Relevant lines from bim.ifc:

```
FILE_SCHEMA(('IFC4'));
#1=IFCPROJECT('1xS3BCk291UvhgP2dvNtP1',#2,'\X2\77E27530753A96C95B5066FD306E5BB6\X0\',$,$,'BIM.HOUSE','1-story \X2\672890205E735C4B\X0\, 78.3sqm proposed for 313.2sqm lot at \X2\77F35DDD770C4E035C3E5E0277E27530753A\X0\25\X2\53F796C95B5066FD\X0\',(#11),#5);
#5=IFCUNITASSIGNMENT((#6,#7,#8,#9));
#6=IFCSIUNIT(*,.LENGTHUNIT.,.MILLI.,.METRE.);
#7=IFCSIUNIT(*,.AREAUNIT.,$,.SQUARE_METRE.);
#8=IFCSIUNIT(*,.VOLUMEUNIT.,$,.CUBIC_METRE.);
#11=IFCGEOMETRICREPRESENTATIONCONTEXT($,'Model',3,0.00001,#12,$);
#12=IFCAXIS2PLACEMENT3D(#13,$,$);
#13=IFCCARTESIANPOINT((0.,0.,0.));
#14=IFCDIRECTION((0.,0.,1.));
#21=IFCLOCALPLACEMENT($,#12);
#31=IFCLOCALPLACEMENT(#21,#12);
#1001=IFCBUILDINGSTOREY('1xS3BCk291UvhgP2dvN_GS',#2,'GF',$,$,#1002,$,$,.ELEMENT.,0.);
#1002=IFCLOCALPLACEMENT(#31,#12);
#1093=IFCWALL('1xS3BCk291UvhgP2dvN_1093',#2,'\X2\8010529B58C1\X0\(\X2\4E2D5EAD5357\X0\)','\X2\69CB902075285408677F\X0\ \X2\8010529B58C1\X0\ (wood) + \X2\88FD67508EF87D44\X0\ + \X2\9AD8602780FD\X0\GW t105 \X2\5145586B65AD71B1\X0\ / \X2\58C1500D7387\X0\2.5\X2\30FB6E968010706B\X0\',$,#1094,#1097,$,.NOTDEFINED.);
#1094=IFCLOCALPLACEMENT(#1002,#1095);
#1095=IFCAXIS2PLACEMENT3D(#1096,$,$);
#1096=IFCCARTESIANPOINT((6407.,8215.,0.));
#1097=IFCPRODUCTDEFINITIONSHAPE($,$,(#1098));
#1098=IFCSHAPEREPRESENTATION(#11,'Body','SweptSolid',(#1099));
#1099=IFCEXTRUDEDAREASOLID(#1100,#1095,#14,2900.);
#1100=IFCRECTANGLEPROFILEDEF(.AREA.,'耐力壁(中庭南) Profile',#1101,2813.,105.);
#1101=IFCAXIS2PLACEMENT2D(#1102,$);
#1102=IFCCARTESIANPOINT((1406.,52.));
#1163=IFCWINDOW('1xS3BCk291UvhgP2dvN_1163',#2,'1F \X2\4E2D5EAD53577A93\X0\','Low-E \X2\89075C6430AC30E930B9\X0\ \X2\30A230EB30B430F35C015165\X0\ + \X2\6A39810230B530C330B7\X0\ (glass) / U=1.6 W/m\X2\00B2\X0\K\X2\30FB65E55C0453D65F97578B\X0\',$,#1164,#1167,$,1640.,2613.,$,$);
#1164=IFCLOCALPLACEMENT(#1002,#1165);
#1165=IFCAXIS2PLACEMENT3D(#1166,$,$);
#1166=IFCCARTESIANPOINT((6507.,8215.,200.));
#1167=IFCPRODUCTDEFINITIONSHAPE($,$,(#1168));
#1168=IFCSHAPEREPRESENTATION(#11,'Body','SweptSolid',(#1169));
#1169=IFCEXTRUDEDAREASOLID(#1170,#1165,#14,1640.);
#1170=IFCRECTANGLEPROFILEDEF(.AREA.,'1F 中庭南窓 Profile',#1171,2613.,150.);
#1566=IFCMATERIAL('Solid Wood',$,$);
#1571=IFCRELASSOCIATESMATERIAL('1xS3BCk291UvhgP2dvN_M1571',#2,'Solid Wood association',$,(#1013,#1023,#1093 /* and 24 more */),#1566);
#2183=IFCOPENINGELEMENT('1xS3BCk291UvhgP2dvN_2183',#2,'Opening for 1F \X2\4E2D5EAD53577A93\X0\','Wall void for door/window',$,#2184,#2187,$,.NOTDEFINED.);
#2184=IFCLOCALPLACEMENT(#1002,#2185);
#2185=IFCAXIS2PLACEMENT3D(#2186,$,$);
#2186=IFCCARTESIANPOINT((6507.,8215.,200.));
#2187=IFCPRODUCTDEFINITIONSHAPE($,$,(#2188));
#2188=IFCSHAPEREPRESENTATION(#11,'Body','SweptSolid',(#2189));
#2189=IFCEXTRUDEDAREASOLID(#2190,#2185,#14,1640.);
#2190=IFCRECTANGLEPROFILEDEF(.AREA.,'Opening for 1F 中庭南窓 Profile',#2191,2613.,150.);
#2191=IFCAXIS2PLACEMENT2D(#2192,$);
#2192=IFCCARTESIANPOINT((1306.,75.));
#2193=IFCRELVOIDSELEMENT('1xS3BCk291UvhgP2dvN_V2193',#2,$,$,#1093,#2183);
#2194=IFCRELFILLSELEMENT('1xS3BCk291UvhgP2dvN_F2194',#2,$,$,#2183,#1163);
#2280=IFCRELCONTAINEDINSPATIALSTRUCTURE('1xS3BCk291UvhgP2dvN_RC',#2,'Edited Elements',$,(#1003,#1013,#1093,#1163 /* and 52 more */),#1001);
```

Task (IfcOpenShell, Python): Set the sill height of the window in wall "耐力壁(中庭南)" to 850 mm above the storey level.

```python
import numpy as np
import ifcopenshell
import ifcopenshell.api.geometry
import ifcopenshell.geom
import ifcopenshell.util.element
import ifcopenshell.util.placement
import ifcopenshell.util.shape
import ifcopenshell.util.unit

model = ifcopenshell.open("bim.ifc")
unit_scale = ifcopenshell.util.unit.calculate_unit_scale(model)

window = model.by_guid("1xS3BCk291UvhgP2dvN_1163")
opening = window.FillsVoids[0].RelatingOpeningElement
storey = ifcopenshell.util.element.get_container(window, ifc_class="IfcBuildingStorey")
level = ifcopenshell.util.placement.get_local_placement(storey.ObjectPlacement)[2, 3]

# The opening's origin need not be at the sill, so measure its lowest point.
shape = ifcopenshell.geom.create_shape(ifcopenshell.geom.settings(), opening)
bottom = ifcopenshell.util.shape.get_shape_bottom_elevation(shape, shape.geometry) / unit_scale
dz = level + 0.85 / unit_scale - bottom

shift = np.array([0.0, 0.0, dz])
# The window is not placed relative to its opening, so move both.
for product in (opening, window):
    matrix = ifcopenshell.util.placement.get_local_placement(product.ObjectPlacement)
    matrix[:3, 3] += shift
    ifcopenshell.api.geometry.edit_object_placement(model, product=product, matrix=matrix, is_si=False)

print(f"moved by {dz * unit_scale:+.3f} m")

model.write("bim_updated.ifc")
```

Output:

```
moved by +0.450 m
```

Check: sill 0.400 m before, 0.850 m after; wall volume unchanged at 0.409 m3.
